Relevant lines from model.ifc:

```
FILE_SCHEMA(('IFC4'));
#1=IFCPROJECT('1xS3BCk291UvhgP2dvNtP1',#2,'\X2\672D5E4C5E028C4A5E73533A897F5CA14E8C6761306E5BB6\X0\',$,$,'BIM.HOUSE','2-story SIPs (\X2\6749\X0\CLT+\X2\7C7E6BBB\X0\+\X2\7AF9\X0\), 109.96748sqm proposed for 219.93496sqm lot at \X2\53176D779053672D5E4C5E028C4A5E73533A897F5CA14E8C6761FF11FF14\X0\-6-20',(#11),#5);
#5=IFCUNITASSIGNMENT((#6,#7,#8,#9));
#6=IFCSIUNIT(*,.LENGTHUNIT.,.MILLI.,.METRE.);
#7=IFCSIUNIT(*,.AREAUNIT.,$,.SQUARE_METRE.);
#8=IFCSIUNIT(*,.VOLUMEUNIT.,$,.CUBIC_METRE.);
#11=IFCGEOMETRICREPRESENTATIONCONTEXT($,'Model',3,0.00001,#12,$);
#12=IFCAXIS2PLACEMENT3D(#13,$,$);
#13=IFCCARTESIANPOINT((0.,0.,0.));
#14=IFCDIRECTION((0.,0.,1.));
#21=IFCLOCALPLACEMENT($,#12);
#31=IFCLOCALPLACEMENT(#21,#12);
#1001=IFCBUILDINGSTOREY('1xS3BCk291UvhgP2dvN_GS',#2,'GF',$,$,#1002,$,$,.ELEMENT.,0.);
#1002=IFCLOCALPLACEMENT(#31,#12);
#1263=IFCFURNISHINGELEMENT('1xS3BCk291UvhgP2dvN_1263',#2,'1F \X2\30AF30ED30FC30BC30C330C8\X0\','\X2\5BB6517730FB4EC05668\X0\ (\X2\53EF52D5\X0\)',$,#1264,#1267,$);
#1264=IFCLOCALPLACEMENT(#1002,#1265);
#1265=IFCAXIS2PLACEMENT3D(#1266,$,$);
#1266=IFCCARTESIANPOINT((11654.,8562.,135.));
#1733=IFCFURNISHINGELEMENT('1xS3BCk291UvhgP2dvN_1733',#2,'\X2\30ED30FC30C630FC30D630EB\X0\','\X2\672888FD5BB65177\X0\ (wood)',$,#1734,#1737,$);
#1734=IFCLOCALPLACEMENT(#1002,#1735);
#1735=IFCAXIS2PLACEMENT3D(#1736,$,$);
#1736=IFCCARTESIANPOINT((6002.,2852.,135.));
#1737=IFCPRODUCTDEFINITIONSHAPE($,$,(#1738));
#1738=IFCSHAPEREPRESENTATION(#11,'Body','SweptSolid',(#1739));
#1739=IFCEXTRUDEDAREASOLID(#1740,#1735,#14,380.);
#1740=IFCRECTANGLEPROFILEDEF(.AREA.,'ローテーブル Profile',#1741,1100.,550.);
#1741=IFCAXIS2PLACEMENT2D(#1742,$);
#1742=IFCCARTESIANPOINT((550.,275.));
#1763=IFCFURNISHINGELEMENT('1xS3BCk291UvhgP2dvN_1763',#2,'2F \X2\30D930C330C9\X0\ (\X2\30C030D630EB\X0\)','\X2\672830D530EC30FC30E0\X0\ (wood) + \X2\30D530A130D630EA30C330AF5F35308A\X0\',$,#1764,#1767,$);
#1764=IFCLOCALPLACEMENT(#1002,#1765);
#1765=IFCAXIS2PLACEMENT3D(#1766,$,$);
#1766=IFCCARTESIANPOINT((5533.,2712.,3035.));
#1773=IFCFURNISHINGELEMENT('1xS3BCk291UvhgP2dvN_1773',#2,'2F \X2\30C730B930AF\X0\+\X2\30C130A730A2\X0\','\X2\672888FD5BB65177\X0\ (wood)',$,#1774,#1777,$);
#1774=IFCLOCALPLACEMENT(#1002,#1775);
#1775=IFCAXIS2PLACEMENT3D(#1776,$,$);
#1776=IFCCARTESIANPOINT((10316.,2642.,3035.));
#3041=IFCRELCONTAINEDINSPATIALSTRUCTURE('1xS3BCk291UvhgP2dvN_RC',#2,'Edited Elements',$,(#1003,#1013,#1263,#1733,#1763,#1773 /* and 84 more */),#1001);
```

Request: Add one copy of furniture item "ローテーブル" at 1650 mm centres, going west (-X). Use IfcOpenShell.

```python
import numpy as np
import ifcopenshell
import ifcopenshell.api.geometry
import ifcopenshell.api.root
import ifcopenshell.util.element
import ifcopenshell.util.placement
import ifcopenshell.util.unit

model = ifcopenshell.open("model.ifc")
unit_scale = ifcopenshell.util.unit.calculate_unit_scale(model)


def reuse_history(source, copy):
    """copy_class also copies each property set's owner history, people and application; keep the originals."""
    for rel in copy.IsDefinedBy:
        if rel.is_a("IfcRelDefinesByProperties") and (history := rel.RelatingPropertyDefinition.OwnerHistory):
            rel.RelatingPropertyDefinition.OwnerHistory = source.OwnerHistory
            ifcopenshell.util.element.remove_deep2(model, history)


source = model.by_guid("1xS3BCk291UvhgP2dvN_1733")
base = ifcopenshell.util.placement.get_local_placement(source.ObjectPlacement)
step = np.array([-1.0, 0.0, 0.0]) * 1.65 / unit_scale

for i in range(1, 2):
    copy = ifcopenshell.api.root.copy_class(model, product=source)
    copy.Representation = ifcopenshell.util.element.copy_deep(
        model, source.Representation, exclude=["IfcGeometricRepresentationContext", "IfcRepresentationMap"]
    )
    reuse_history(source, copy)
    matrix = base.copy()
    matrix[:3, 3] += i * step
    print("added at", matrix[:3, 3].round(3) + 0.0)
    ifcopenshell.api.geometry.edit_object_placement(model, product=copy, matrix=matrix, is_si=False)

model.write("model_updated.ifc")
```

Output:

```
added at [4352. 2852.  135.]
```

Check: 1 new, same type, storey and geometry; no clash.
